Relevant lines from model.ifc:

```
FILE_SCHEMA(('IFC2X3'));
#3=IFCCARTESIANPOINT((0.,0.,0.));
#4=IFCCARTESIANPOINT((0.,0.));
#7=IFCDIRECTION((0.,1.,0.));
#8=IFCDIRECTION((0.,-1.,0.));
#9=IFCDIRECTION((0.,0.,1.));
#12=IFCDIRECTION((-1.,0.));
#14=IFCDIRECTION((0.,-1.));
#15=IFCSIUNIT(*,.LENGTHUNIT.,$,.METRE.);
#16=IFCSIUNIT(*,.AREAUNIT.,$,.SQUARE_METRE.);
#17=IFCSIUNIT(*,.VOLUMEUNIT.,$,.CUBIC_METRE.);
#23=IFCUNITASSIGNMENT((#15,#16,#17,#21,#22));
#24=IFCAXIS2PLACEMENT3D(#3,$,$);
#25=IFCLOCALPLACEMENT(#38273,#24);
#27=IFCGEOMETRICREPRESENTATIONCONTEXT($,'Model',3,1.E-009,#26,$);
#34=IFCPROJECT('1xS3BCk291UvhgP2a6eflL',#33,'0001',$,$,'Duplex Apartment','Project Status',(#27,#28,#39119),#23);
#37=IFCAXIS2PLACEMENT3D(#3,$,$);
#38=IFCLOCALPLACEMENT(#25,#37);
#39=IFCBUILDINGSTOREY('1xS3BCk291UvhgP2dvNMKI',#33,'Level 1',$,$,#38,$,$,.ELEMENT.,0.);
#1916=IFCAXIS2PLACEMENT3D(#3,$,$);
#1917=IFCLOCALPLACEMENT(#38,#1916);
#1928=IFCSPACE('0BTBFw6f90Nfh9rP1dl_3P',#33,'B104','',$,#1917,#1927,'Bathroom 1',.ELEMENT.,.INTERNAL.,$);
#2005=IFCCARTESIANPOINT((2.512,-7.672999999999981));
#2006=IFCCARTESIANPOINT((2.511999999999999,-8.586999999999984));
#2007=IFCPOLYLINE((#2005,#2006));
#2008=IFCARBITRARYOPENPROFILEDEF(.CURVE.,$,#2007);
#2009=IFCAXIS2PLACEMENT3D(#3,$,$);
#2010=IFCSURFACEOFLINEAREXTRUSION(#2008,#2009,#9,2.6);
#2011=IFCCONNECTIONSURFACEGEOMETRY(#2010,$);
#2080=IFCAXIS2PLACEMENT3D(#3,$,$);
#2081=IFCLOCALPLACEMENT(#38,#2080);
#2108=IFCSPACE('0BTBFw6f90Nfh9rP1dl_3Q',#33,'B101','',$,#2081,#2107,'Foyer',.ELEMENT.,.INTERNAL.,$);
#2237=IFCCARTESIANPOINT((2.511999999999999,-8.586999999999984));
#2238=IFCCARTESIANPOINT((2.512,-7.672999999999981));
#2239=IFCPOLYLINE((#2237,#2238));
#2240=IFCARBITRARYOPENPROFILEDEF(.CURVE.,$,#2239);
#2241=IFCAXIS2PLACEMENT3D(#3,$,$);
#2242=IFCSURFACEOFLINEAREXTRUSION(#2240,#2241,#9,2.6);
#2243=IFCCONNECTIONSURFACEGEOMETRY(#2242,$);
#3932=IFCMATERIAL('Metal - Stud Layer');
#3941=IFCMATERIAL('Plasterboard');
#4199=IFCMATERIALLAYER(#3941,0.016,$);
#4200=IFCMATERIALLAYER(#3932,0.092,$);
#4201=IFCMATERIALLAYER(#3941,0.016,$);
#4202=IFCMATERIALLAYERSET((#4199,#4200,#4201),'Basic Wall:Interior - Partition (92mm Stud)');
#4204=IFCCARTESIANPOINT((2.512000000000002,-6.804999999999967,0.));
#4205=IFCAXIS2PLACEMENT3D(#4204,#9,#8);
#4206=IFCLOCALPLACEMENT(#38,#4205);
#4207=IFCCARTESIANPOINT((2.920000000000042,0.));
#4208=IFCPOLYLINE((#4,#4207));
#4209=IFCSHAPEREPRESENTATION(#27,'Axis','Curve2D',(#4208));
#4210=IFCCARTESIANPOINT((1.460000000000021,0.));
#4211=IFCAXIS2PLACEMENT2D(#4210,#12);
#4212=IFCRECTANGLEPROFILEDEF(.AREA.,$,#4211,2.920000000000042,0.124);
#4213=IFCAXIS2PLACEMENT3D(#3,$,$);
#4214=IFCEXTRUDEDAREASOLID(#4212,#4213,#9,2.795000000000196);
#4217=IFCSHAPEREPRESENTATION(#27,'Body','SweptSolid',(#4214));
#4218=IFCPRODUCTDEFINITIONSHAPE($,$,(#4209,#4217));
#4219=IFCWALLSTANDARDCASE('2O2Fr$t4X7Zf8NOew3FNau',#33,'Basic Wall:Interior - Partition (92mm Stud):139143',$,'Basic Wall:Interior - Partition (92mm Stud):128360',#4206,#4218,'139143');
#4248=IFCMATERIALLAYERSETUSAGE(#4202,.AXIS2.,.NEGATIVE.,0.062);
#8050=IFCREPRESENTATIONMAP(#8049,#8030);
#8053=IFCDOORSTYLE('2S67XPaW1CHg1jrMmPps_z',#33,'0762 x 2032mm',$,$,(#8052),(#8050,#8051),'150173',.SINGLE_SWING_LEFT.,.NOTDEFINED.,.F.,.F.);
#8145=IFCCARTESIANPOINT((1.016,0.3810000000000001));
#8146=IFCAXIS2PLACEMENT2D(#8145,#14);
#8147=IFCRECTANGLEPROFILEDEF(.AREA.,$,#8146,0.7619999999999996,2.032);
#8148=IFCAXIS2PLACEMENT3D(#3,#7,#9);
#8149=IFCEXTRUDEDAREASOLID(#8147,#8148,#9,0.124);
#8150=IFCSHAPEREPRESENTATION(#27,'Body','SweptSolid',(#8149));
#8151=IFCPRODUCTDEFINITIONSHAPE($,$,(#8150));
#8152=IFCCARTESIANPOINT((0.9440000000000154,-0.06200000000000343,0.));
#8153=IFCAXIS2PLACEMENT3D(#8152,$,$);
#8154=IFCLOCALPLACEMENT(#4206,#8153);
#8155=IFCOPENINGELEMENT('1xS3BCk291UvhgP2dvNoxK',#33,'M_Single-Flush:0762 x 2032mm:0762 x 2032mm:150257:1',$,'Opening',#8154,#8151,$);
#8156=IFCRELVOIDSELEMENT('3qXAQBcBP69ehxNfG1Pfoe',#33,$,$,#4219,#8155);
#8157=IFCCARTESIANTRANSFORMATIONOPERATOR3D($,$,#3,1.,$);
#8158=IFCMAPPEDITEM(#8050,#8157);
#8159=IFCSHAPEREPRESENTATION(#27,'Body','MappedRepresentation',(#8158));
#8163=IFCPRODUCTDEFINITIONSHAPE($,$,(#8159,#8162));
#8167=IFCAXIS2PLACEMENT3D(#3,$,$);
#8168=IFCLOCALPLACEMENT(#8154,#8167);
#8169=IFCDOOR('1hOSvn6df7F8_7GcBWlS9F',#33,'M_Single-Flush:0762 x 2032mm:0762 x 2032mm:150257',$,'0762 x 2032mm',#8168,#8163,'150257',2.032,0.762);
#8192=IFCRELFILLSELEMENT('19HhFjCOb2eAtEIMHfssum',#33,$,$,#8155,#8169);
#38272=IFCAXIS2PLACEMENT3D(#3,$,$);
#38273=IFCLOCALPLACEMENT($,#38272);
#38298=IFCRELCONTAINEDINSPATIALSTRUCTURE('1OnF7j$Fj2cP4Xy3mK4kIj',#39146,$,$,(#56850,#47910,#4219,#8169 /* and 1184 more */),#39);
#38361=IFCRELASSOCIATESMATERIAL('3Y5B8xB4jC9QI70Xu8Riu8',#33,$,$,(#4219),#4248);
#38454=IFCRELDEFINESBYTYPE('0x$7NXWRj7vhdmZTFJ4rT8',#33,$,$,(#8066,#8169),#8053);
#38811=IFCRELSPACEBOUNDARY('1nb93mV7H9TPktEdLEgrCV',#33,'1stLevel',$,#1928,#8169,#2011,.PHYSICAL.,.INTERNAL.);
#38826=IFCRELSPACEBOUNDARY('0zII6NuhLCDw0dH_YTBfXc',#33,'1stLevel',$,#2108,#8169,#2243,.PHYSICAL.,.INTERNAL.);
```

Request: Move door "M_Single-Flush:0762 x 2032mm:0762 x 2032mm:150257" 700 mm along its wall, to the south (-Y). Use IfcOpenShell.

```python
import numpy as np
import ifcopenshell
import ifcopenshell.api.geometry
import ifcopenshell.util.placement

model = ifcopenshell.open("model.ifc")

door = model.by_guid("1hOSvn6df7F8_7GcBWlS9F")
opening = door.FillsVoids[0].RelatingOpeningElement
wall = opening.VoidsElements[0].RelatingBuildingElement

wall_matrix = ifcopenshell.util.placement.get_local_placement(wall.ObjectPlacement)
shift = wall_matrix[:3, 0] * 0.7
before = ifcopenshell.util.placement.get_local_placement(door.ObjectPlacement)[:3, 3].copy()

# The door is placed relative to its opening, so it follows when the opening moves.
matrix = ifcopenshell.util.placement.get_local_placement(opening.ObjectPlacement)
matrix[:3, 3] += shift
ifcopenshell.api.geometry.edit_object_placement(
    model, product=opening, matrix=matrix, is_si=False, should_transform_children=True
)

# Space boundary surfaces are stored in each space's coordinates; move them too.
for rel in door.ProvidesBoundaries:
    if not rel.ConnectionGeometry:
        continue
    surface = rel.ConnectionGeometry.SurfaceOnRelatingElement
    space_matrix = ifcopenshell.util.placement.get_local_placement(rel.RelatingSpace.ObjectPlacement)
    point = np.array(surface.Position.Location.Coordinates) + space_matrix[:3, :3].T @ shift
    surface.Position = model.createIfcAxis2Placement3D(
        model.createIfcCartesianPoint(point.tolist()), surface.Position.Axis, surface.Position.RefDirection
    )

after = ifcopenshell.util.placement.get_local_placement(door.ObjectPlacement)[:3, 3]
print("door moved by", (after - before).round(3) + 0.0)

model.write("model_updated.ifc")
```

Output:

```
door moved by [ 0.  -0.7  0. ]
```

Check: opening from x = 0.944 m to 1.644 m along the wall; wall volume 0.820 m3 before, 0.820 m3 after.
